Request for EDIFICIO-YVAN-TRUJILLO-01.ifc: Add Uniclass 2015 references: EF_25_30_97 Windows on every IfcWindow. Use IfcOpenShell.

First a look at what the model holds.

```python
import ifcopenshell

model = ifcopenshell.open("EDIFICIO-YVAN-TRUJILLO-01.ifc")
print(model.schema)
print("classifications:", [c.Name for c in model.by_type("IfcClassification")])
for ifc_class in ("IfcDoor", "IfcRoof", "IfcStair", "IfcWall", "IfcWindow"):
    print(ifc_class, len(model.by_type(ifc_class)))
```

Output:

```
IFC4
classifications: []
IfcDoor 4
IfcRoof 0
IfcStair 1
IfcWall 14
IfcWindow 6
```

```python
import ifcopenshell
import ifcopenshell.api.classification

model = ifcopenshell.open("EDIFICIO-YVAN-TRUJILLO-01.ifc")

system = ifcopenshell.api.classification.add_classification(model, classification="Uniclass 2015")

codes = {
    "IfcWindow": ("EF_25_30_97", "Windows"),
}
for ifc_class, (code, name) in codes.items():
    products = model.by_type(ifc_class)
    ifcopenshell.api.classification.add_reference(
        model, products=products, classification=system, identification=code, name=name
    )
    print(code, len(products))

model.write("EDIFICIO-YVAN-TRUJILLO-01_updated.ifc")
```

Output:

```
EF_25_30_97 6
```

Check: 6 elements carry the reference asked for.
